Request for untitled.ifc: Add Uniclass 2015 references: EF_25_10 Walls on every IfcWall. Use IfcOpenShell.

First a look at what the model holds.

```python
import ifcopenshell

model = ifcopenshell.open("untitled.ifc")
print(model.schema)
print("classifications:", [c.Name for c in model.by_type("IfcClassification")])
for ifc_class in ("IfcDoor", "IfcRoof", "IfcStair", "IfcWall", "IfcWindow"):
    print(ifc_class, len(model.by_type(ifc_class)))
```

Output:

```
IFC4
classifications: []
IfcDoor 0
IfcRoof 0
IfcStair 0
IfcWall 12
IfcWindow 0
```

```python
import ifcopenshell
import ifcopenshell.api.classification

model = ifcopenshell.open("untitled.ifc")

system = ifcopenshell.api.classification.add_classification(model, classification="Uniclass 2015")

codes = {
    "IfcWall": ("EF_25_10", "Walls"),
}
for ifc_class, (code, name) in codes.items():
    products = model.by_type(ifc_class)
    ifcopenshell.api.classification.add_reference(
        model, products=products, classification=system, identification=code, name=name
    )
    print(code, len(products))

model.write("untitled-out.ifc")
```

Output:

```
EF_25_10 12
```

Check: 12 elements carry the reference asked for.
